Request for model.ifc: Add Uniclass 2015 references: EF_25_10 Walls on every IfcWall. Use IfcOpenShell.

First a look at what the model holds.

```python
import ifcopenshell

model = ifcopenshell.open("model.ifc")
print(model.schema)
print("classifications:", [c.Name for c in model.by_type("IfcClassification")])
for ifc_class in ("IfcDoor", "IfcRoof", "IfcStair", "IfcWall", "IfcWindow"):
    print(ifc_class, len(model.by_type(ifc_class)))
```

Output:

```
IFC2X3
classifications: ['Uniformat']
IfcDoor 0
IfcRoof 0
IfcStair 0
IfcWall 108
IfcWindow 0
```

```python
import ifcopenshell
import ifcopenshell.api.classification

model = ifcopenshell.open("model.ifc")

# IFC2X3 requires Source and Edition and has no link from the project to the system.
system = model.create_entity("IfcClassification", Source="NBS", Edition="2015", Name="Uniclass 2015")

codes = {
    "IfcWall": ("EF_25_10", "Walls"),
}
for ifc_class, (code, name) in codes.items():
    products = model.by_type(ifc_class)
    ifcopenshell.api.classification.add_reference(
        model, products=products, classification=system, identification=code, name=name
    )
    print(code, len(products))

model.write("model-out.ifc")
```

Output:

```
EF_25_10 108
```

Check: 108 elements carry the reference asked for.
